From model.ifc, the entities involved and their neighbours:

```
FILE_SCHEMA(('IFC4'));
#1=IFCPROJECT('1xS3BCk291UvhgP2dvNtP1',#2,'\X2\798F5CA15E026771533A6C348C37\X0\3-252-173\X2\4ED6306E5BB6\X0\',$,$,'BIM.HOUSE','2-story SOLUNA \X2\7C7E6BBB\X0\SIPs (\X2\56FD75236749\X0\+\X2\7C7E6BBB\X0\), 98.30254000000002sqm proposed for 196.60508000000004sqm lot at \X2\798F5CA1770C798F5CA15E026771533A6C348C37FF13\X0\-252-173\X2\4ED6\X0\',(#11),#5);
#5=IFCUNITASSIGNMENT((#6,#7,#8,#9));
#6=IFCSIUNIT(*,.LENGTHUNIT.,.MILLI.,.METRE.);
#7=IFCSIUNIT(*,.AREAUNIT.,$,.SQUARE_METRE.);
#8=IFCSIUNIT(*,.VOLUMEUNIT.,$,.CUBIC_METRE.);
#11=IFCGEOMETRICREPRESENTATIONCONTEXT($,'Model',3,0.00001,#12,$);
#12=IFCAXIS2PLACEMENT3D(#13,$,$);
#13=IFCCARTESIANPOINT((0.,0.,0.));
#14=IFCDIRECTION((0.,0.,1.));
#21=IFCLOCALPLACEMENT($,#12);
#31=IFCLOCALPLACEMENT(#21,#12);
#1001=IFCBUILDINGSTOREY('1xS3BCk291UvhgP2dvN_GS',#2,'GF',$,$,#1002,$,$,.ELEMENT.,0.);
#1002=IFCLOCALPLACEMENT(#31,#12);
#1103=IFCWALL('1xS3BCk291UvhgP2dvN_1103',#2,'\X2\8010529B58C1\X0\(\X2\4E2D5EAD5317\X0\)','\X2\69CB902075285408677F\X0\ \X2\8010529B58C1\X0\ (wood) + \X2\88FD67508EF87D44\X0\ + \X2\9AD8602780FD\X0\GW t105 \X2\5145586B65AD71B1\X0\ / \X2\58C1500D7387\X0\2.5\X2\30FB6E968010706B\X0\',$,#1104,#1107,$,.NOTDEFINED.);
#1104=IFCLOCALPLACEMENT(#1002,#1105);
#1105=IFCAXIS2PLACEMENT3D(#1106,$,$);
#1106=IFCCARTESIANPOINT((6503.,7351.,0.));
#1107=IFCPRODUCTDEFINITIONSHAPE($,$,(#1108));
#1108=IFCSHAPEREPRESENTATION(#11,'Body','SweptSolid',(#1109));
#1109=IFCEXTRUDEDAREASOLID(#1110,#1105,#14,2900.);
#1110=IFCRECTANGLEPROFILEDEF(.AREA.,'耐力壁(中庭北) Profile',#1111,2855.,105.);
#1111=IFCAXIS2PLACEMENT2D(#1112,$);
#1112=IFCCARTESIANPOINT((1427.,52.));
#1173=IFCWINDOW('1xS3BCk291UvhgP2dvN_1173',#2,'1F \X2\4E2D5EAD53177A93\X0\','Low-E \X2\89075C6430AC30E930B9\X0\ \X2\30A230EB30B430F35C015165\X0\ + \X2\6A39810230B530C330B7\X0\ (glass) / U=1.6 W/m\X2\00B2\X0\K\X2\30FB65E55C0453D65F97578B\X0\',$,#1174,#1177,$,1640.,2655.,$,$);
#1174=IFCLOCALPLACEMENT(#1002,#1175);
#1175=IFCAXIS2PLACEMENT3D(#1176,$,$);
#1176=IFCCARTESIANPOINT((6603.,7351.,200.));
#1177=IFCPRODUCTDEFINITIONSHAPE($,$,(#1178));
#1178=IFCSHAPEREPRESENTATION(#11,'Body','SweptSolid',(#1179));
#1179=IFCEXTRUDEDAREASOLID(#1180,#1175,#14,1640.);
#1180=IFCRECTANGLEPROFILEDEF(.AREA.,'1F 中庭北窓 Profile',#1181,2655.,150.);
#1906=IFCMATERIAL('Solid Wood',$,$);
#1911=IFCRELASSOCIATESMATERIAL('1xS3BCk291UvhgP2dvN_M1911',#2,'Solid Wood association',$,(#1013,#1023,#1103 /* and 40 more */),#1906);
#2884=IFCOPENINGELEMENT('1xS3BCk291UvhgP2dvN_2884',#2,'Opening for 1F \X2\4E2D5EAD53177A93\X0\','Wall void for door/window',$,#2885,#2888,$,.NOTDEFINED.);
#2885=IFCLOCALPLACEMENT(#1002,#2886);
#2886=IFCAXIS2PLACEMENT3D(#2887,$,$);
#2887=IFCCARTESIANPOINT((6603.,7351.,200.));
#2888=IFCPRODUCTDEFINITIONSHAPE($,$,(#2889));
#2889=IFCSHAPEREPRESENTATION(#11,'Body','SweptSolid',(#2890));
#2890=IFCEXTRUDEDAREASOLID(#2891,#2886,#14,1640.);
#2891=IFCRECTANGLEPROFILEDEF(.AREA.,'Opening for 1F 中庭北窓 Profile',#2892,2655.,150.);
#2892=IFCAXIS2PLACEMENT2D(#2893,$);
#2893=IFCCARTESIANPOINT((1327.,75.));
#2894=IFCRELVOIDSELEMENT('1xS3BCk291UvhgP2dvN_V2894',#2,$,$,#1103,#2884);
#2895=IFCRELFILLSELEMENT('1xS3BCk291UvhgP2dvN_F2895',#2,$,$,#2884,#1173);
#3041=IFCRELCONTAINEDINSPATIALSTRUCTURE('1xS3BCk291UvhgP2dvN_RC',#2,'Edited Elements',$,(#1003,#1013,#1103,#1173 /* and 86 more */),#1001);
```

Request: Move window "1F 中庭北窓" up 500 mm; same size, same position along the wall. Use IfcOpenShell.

```python
import numpy as np
import ifcopenshell
import ifcopenshell.api.geometry
import ifcopenshell.util.placement
import ifcopenshell.util.unit

model = ifcopenshell.open("model.ifc")
unit_scale = ifcopenshell.util.unit.calculate_unit_scale(model)

window = model.by_id(1173)
opening = window.FillsVoids[0].RelatingOpeningElement
dz = 500.0

shift = np.array([0.0, 0.0, dz])
# The window is not placed relative to its opening, so move both.
for product in (opening, window):
    matrix = ifcopenshell.util.placement.get_local_placement(product.ObjectPlacement)
    matrix[:3, 3] += shift
    ifcopenshell.api.geometry.edit_object_placement(model, product=product, matrix=matrix, is_si=False)

print(f"moved by {dz * unit_scale:+.3f} m")

model.write("model_rev.ifc")
```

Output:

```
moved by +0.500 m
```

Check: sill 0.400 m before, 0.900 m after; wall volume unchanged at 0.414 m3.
